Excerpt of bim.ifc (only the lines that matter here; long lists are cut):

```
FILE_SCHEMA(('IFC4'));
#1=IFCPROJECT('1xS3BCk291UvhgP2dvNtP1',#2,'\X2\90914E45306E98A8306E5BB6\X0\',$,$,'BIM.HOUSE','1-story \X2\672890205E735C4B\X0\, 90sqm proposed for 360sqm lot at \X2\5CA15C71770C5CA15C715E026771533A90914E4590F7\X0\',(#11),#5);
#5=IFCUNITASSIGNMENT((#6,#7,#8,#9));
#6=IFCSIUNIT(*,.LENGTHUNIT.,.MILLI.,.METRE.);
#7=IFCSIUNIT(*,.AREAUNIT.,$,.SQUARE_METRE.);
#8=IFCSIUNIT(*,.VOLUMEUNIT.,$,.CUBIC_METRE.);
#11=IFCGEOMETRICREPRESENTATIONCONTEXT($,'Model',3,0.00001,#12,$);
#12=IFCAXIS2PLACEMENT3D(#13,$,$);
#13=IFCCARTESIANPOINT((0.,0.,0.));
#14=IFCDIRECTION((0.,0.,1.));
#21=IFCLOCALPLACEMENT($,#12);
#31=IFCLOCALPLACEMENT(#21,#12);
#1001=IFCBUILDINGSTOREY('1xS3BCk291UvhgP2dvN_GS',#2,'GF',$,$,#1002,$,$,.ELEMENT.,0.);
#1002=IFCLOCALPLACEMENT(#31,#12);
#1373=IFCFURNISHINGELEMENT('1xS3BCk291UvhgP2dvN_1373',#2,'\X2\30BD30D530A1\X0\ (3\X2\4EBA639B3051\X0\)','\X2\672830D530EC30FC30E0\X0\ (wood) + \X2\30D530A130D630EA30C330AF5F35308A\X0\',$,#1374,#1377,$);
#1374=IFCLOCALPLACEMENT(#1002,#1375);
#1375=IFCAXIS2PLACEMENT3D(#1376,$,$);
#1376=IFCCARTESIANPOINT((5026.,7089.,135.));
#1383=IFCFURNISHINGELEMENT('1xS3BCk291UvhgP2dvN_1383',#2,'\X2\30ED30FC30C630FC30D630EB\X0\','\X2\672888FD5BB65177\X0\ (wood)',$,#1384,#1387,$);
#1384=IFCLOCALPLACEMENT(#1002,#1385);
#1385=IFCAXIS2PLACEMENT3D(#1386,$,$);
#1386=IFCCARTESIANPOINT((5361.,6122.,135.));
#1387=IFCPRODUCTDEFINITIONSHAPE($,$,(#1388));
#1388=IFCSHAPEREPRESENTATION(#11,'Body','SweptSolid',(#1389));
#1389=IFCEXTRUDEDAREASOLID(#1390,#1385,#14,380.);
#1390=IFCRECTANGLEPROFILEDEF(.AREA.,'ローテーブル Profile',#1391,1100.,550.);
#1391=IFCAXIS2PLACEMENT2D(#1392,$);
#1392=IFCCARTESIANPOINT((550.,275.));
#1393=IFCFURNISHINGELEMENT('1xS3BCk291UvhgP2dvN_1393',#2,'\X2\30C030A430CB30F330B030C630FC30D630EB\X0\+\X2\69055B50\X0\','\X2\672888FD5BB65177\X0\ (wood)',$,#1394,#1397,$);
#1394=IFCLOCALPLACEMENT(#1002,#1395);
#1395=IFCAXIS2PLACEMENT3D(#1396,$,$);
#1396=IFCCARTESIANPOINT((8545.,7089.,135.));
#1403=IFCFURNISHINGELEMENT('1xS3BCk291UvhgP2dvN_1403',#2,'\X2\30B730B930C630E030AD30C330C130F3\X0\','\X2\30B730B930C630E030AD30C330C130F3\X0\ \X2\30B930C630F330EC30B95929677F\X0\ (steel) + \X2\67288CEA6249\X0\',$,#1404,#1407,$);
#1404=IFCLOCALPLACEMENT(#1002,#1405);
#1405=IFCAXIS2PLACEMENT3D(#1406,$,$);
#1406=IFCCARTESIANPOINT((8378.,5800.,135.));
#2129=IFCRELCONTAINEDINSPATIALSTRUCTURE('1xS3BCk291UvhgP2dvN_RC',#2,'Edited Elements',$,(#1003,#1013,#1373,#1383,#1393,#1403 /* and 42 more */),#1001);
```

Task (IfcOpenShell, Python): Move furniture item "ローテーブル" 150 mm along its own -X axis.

```python
import ifcopenshell
import ifcopenshell.api.geometry
import ifcopenshell.util.placement

model = ifcopenshell.open("bim.ifc")

item = model.by_guid("1xS3BCk291UvhgP2dvN_1383")
matrix = ifcopenshell.util.placement.get_local_placement(item.ObjectPlacement)
matrix[:3, 3] -= matrix[:3, 0] * 150.0
ifcopenshell.api.geometry.edit_object_placement(model, product=item, matrix=matrix, is_si=False)

print(ifcopenshell.util.placement.get_local_placement(item.ObjectPlacement).round(3) + 0.0)

model.write("bim_rev.ifc")
```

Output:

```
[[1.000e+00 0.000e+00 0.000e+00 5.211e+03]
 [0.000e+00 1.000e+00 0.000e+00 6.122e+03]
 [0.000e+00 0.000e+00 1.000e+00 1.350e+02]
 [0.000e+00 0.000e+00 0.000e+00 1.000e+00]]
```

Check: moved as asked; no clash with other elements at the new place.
